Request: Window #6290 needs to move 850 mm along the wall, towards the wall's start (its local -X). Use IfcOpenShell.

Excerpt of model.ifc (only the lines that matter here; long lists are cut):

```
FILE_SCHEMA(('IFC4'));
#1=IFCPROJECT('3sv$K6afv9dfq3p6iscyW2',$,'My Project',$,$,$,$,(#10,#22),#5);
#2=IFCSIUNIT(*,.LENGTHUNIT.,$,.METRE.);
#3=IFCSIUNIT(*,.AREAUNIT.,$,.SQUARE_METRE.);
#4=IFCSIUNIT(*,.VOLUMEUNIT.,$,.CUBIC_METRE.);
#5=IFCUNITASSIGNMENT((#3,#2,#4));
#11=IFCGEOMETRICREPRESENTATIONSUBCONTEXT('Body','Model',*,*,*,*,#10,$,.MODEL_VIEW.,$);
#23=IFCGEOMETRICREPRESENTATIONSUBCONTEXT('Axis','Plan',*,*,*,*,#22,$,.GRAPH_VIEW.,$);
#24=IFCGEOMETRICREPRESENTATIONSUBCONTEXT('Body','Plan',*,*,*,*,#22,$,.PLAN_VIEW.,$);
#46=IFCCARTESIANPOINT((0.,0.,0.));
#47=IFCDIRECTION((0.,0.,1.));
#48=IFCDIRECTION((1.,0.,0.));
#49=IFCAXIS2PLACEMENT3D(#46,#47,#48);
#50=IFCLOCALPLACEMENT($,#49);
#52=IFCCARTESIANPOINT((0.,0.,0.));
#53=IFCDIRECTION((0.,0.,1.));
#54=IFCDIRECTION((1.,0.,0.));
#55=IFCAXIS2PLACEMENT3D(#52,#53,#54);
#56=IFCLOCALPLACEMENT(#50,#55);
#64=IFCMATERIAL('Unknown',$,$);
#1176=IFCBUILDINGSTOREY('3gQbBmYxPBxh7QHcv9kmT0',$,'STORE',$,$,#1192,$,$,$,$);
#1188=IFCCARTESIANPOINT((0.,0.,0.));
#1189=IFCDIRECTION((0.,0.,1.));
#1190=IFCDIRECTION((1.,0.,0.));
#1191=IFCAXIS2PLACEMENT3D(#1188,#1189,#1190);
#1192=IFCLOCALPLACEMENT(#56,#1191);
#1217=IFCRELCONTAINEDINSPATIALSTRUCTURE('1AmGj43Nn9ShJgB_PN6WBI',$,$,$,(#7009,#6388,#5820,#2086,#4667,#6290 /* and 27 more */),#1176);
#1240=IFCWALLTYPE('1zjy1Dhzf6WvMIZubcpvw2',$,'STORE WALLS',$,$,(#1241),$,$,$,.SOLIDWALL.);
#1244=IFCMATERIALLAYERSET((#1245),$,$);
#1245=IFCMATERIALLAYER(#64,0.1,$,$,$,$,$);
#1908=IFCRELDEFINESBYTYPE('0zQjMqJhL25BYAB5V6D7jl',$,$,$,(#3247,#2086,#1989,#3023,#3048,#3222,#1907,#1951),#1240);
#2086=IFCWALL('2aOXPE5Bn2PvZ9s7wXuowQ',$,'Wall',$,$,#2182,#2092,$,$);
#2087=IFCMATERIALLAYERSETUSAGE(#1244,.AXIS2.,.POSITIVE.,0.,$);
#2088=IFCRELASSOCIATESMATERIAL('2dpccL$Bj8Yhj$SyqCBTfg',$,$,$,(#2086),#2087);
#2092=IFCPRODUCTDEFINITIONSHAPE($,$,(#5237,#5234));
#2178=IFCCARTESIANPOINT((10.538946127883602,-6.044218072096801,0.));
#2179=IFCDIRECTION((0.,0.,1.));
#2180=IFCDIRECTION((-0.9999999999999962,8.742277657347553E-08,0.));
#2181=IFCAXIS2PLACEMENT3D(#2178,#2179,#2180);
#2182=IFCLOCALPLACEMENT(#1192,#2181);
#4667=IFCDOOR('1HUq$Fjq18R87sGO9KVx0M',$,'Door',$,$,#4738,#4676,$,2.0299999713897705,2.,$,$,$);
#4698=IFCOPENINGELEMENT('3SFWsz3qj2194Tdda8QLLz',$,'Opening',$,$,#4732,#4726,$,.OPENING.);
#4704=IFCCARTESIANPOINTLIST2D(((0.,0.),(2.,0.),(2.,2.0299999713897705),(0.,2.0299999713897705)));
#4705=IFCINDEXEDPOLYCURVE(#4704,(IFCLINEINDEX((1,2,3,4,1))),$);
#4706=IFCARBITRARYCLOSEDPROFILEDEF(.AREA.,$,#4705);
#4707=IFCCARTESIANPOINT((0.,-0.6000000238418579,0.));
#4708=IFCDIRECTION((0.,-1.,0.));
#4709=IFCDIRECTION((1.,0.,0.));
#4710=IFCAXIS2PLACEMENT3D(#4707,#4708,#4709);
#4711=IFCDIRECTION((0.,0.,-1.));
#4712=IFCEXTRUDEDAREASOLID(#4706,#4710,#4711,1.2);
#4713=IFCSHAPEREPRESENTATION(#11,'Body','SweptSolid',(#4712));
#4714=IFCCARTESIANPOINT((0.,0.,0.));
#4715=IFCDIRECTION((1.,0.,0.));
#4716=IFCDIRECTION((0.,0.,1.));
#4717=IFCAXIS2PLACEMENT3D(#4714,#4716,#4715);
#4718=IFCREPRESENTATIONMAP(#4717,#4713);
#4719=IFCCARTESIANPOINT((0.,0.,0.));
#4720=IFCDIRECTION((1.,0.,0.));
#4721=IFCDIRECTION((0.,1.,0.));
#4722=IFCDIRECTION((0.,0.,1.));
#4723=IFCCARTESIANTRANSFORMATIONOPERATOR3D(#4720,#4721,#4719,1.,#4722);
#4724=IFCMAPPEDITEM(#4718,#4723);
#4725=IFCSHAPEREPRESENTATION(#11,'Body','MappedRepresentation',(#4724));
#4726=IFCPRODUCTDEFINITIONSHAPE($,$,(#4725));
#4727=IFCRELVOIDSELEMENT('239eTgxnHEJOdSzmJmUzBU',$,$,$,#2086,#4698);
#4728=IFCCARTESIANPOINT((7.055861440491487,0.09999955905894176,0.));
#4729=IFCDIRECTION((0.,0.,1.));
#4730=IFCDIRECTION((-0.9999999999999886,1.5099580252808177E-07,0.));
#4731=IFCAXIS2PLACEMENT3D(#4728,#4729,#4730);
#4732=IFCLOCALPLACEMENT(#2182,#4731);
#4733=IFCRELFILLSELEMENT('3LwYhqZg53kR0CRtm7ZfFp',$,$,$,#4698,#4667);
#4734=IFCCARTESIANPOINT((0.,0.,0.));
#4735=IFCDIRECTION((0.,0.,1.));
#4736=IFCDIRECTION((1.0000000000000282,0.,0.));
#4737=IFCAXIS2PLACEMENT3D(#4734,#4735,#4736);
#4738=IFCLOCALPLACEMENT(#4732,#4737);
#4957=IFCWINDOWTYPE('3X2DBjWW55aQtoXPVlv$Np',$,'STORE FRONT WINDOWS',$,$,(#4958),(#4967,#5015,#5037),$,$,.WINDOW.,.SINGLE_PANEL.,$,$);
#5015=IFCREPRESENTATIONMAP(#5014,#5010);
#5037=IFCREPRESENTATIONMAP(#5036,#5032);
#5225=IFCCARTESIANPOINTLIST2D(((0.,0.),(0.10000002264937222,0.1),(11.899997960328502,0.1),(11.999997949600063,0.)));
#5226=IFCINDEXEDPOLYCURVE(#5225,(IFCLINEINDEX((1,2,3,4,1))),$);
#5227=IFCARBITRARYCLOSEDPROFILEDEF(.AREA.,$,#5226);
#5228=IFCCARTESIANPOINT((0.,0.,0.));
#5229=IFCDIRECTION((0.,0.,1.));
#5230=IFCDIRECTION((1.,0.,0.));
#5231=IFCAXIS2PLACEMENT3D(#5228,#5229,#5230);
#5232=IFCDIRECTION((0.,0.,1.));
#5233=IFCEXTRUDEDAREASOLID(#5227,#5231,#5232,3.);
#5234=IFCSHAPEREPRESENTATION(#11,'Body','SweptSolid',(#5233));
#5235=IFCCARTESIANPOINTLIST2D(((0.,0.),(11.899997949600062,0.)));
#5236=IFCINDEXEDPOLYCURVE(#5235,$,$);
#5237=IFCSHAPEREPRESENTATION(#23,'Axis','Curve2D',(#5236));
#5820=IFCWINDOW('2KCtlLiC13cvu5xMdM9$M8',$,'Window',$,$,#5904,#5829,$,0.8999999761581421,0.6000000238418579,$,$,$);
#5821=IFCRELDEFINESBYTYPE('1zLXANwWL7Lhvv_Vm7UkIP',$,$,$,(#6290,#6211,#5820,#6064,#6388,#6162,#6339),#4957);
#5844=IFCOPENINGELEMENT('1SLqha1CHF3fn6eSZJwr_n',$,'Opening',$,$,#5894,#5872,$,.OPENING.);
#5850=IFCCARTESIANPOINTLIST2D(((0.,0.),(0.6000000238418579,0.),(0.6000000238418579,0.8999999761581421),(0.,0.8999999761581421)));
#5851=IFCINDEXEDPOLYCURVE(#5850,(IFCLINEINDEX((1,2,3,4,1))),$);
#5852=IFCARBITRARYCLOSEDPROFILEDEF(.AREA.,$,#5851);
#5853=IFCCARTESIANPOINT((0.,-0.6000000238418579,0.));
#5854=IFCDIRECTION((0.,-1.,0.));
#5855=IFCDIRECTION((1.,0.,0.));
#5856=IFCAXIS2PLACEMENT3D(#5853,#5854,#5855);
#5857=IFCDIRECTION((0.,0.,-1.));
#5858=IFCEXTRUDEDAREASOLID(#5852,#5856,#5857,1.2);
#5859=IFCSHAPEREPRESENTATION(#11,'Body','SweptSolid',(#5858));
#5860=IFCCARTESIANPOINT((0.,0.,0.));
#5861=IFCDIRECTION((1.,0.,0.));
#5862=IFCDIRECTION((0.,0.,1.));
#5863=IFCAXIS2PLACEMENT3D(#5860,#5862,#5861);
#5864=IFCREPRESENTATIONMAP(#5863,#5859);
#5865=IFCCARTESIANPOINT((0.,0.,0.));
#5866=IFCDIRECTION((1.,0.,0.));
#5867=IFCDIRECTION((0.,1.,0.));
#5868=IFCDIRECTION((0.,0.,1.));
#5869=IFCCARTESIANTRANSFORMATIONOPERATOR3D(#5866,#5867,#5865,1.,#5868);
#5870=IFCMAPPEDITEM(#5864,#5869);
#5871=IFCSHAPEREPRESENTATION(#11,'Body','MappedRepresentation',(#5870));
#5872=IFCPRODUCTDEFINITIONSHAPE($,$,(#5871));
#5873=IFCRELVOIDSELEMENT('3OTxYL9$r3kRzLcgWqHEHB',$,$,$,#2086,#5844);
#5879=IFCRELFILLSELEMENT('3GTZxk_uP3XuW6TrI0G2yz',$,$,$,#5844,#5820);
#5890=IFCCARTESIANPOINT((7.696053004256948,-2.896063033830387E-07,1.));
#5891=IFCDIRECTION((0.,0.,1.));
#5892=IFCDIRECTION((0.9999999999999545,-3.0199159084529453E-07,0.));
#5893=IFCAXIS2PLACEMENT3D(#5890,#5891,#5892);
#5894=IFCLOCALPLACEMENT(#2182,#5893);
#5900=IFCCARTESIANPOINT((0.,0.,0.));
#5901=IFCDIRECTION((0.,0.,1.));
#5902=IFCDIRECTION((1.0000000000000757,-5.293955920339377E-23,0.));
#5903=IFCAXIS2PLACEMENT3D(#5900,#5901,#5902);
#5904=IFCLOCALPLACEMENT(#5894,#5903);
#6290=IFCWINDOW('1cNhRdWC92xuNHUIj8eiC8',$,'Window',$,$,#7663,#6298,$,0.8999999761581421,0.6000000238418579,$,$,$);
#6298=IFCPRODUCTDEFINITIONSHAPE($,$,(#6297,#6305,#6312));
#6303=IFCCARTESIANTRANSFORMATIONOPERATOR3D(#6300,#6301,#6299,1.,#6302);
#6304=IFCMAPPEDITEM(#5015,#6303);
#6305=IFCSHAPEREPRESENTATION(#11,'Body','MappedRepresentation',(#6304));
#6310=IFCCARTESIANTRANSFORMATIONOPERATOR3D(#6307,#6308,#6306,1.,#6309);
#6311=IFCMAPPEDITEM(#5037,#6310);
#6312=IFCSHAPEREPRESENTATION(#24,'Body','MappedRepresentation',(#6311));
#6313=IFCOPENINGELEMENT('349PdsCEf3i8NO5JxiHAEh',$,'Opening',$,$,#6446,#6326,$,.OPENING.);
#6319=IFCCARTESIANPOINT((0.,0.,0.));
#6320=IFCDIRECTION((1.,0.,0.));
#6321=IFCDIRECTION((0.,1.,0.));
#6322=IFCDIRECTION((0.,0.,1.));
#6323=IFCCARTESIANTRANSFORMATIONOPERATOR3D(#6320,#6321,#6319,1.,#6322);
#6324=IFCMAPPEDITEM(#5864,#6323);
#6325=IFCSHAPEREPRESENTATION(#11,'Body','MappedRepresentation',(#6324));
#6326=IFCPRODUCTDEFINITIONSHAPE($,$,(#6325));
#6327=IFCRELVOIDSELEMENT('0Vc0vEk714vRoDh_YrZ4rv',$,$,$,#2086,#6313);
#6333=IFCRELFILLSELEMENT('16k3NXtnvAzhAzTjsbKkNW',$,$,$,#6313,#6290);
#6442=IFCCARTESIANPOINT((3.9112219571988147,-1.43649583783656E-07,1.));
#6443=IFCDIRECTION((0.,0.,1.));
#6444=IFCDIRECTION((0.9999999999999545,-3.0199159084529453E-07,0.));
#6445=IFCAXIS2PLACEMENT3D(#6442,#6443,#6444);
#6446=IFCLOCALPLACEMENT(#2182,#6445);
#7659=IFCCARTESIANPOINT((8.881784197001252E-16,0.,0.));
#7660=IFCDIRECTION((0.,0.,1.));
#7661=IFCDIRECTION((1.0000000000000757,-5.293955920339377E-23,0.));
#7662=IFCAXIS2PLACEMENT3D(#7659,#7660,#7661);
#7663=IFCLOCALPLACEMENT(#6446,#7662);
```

```python
import ifcopenshell
import ifcopenshell.api.geometry
import ifcopenshell.util.placement
import ifcopenshell.util.unit

model = ifcopenshell.open("model.ifc")
unit_scale = ifcopenshell.util.unit.calculate_unit_scale(model)

window = model.by_guid("1cNhRdWC92xuNHUIj8eiC8")
opening = window.FillsVoids[0].RelatingOpeningElement
wall = opening.VoidsElements[0].RelatingBuildingElement

wall_matrix = ifcopenshell.util.placement.get_local_placement(wall.ObjectPlacement)
shift = wall_matrix[:3, 0] * -0.85 / unit_scale
before = ifcopenshell.util.placement.get_local_placement(window.ObjectPlacement)[:3, 3].copy()

# The window is placed relative to its opening, so it follows when the opening moves.
matrix = ifcopenshell.util.placement.get_local_placement(opening.ObjectPlacement)
matrix[:3, 3] += shift
ifcopenshell.api.geometry.edit_object_placement(
    model, product=opening, matrix=matrix, is_si=False, should_transform_children=True
)

after = ifcopenshell.util.placement.get_local_placement(window.ObjectPlacement)[:3, 3]
print("window moved by", (after - before).round(3) + 0.0)

model.write("model-out.ifc")
```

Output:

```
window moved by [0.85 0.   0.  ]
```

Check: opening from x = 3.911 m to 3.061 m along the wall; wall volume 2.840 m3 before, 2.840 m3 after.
